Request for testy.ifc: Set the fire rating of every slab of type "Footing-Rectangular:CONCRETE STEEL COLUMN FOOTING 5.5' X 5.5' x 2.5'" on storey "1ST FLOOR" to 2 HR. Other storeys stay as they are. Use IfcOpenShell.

First a look at what the model holds.

```python
import ifcopenshell
import ifcopenshell.util.element

model = ifcopenshell.open("testy.ifc")
print(model.schema)
storey = next(s for s in model.by_type("IfcBuildingStorey") if s.Name == "1ST FLOOR")
slabs = [e for e in ifcopenshell.util.element.get_decomposition(storey) if e.is_a("IfcSlab")]
seen = {}
for e in slabs:
    element_type = ifcopenshell.util.element.get_type(e)
    key = (element_type.Name if element_type != e and element_type else None, ifcopenshell.util.element.get_pset(e, "Pset_SlabCommon", "FireRating"))
    seen[key] = seen.get(key, 0) + 1
for (name, value), count in sorted(seen.items(), key=str):
    print(count, "x", name, "|", value)
```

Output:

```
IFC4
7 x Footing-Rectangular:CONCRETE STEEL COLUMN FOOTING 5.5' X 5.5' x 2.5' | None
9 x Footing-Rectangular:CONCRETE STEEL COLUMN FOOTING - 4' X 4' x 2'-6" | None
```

```python
import ifcopenshell
import ifcopenshell.api.pset
import ifcopenshell.util.element

model = ifcopenshell.open("testy.ifc")

storey = next(s for s in model.by_type("IfcBuildingStorey") if s.Name == "1ST FLOOR")
slabs = [e for e in ifcopenshell.util.element.get_decomposition(storey) if e.is_a("IfcSlab")]

count = 0
for e in slabs:
    element_type = ifcopenshell.util.element.get_type(e)
    if element_type in (None, e) or element_type.Name != "Footing-Rectangular:CONCRETE STEEL COLUMN FOOTING 5.5' X 5.5' x 2.5'":
        continue
    # add_pset returns the element's existing set when there is one.
    pset = ifcopenshell.api.pset.add_pset(model, product=e, name="Pset_SlabCommon")
    ifcopenshell.api.pset.edit_pset(model, pset=pset, properties={"FireRating": "2 HR"})
    count += 1

print(count, "slabs updated")

model.write("testy_edited.ifc")
```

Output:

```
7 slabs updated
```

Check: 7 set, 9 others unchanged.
